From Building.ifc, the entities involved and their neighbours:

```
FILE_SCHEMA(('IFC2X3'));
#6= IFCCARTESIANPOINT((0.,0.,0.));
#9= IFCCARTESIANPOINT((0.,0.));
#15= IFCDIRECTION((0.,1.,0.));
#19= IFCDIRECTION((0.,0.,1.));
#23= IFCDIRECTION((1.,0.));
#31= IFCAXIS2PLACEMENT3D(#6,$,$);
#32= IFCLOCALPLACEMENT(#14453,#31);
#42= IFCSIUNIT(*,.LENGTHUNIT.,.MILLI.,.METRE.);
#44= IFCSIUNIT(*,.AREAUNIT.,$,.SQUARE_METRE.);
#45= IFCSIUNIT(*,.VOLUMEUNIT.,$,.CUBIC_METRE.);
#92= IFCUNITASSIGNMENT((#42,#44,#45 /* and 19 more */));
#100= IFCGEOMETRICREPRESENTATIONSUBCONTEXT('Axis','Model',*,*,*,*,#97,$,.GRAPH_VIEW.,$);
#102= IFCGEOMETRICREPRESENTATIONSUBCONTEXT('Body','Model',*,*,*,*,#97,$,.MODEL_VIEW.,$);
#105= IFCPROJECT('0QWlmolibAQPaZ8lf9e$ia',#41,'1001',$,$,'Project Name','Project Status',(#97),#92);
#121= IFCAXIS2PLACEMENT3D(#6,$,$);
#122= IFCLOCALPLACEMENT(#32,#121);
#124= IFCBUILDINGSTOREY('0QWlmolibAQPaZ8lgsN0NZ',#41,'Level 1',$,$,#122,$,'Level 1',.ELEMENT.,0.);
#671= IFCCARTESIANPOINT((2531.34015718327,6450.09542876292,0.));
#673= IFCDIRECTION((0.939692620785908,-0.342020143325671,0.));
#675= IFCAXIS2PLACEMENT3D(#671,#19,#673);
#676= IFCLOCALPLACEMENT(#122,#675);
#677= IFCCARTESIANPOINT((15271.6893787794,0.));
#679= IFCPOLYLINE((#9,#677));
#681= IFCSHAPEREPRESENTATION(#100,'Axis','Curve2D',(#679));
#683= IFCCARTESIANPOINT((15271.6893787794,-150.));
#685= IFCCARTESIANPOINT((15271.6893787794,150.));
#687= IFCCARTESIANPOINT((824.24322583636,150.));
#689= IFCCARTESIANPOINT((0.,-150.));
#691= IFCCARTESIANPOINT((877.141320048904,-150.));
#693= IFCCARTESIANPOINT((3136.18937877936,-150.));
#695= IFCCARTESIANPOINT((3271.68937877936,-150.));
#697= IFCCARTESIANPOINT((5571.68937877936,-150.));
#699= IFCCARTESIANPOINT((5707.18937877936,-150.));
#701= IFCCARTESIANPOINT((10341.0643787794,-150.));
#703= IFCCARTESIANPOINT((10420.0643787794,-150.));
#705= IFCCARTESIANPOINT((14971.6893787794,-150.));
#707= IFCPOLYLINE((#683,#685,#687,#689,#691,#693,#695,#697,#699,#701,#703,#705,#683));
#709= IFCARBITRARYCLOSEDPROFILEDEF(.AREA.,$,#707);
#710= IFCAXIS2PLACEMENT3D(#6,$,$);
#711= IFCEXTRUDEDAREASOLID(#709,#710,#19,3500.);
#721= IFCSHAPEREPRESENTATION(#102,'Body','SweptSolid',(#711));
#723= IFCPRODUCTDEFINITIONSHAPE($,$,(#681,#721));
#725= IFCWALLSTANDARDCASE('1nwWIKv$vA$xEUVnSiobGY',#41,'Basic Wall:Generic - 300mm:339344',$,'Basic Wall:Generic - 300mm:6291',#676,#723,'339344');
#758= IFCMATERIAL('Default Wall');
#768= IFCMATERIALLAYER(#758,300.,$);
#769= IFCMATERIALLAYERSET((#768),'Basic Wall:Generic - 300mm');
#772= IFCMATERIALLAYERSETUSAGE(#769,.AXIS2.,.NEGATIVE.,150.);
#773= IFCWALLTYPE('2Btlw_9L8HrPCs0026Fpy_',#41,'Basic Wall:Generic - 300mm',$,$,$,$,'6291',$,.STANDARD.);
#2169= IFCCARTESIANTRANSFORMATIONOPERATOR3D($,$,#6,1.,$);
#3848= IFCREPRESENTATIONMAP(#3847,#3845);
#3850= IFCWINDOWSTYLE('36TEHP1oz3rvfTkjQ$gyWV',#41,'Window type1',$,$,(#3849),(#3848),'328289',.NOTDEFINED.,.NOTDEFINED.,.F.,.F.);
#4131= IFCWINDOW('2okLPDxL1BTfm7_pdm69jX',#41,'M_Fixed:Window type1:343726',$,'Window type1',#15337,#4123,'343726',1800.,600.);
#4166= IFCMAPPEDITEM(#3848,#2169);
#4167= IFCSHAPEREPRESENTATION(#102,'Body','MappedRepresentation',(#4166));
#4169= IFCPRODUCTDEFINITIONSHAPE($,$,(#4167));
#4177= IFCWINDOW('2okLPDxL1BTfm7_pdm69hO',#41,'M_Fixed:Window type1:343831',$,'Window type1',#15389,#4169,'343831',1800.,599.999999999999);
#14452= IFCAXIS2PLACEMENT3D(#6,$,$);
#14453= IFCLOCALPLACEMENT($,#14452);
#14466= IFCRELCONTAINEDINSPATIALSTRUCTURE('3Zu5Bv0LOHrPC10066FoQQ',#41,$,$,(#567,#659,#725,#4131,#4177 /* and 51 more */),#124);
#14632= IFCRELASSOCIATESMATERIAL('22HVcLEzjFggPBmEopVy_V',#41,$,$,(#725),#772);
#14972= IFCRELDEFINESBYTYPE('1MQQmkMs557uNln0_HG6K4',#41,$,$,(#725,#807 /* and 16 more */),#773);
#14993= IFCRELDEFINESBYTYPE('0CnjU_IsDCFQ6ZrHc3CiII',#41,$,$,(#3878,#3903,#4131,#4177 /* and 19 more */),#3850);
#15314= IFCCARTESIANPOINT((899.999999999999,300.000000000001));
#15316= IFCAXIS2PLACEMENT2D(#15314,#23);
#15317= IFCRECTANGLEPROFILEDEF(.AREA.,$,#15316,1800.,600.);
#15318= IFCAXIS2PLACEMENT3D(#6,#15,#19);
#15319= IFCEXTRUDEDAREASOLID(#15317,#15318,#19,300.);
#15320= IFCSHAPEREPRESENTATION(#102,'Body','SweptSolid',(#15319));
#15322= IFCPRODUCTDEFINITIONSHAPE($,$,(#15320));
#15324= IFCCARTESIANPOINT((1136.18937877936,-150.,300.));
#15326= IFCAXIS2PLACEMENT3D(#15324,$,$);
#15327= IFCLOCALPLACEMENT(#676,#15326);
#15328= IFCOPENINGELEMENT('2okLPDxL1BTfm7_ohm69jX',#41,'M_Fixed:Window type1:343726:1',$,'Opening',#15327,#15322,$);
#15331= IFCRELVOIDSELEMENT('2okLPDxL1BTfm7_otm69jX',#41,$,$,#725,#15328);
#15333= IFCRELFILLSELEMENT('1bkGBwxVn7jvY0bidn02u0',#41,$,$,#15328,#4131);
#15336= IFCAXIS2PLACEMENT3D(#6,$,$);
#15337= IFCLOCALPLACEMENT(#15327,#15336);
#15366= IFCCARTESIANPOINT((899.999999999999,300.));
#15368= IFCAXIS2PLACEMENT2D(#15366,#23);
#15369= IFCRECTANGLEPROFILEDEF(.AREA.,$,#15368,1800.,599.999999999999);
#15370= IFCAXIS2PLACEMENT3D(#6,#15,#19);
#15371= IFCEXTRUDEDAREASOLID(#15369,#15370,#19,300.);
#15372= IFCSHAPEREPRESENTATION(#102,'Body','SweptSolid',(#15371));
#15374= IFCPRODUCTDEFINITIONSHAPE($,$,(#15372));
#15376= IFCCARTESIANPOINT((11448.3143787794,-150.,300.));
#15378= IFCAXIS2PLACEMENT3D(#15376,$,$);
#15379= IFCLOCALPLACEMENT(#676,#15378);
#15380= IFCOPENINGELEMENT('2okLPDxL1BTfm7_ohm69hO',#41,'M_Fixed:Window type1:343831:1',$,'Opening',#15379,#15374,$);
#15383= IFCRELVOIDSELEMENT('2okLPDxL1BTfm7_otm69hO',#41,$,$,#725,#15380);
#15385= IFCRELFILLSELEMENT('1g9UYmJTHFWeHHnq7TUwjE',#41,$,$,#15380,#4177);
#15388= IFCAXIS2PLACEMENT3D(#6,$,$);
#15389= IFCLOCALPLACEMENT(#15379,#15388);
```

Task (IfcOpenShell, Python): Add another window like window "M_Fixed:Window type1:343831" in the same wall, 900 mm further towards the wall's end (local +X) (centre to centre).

```python
import ifcopenshell
import ifcopenshell.api.feature
import ifcopenshell.api.geometry
import ifcopenshell.api.root
import ifcopenshell.geom
import ifcopenshell.util.element
import ifcopenshell.util.placement
import ifcopenshell.util.shape
import ifcopenshell.util.unit

model = ifcopenshell.open("Building.ifc")
unit_scale = ifcopenshell.util.unit.calculate_unit_scale(model)
settings = ifcopenshell.geom.settings()


def volume(element):
    """Net volume in cubic metres, openings subtracted."""
    shape = ifcopenshell.geom.create_shape(settings, element)
    return ifcopenshell.util.shape.get_volume(shape.geometry)


def reuse_history(source, copy):
    """copy_class also copies each property set's owner history, people and application; keep the originals."""
    for rel in copy.IsDefinedBy:
        if rel.is_a("IfcRelDefinesByProperties") and (history := rel.RelatingPropertyDefinition.OwnerHistory):
            rel.RelatingPropertyDefinition.OwnerHistory = source.OwnerHistory
            ifcopenshell.util.element.remove_deep2(model, history)


window = model.by_id(4177)
opening = window.FillsVoids[0].RelatingOpeningElement
wall = opening.VoidsElements[0].RelatingBuildingElement
before = volume(wall)
shift = ifcopenshell.util.placement.get_local_placement(wall.ObjectPlacement)[:3, 0] * 0.9 / unit_scale

# copy_class copies the void relationship, type, container and properties, but no geometry.
new_opening = ifcopenshell.api.root.copy_class(model, product=opening)
new_opening.Representation = ifcopenshell.util.element.copy_deep(
    model, opening.Representation, exclude=["IfcGeometricRepresentationContext", "IfcRepresentationMap"]
)
new_opening.Name = "M_Fixed:Window type1"
new_window = ifcopenshell.api.root.copy_class(model, product=window)
new_window.Representation = ifcopenshell.util.element.copy_deep(
    model, window.Representation, exclude=["IfcGeometricRepresentationContext", "IfcRepresentationMap"]
)
new_window.Name = "M_Fixed:Window type1"
new_window.Tag = None
reuse_history(window, new_window)
fills = ifcopenshell.api.feature.add_filling(model, opening=new_opening, element=new_window)
fills.OwnerHistory = new_window.OwnerHistory  # required in IFC2X3

for old, new in ((opening, new_opening), (window, new_window)):
    matrix = ifcopenshell.util.placement.get_local_placement(old.ObjectPlacement)
    matrix[:3, 3] += shift
    ifcopenshell.api.geometry.edit_object_placement(model, product=new, matrix=matrix, is_si=False)

after = volume(wall)

print(f"wall volume {before:.3f} -> {after:.3f} m3")

model.write("Building_edited.ifc")
```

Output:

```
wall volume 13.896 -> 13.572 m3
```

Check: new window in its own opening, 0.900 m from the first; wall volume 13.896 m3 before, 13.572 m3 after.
